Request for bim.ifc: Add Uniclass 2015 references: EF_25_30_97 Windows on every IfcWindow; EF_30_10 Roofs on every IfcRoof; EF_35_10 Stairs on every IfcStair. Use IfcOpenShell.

First a look at what the model holds.

```python
import ifcopenshell

model = ifcopenshell.open("bim.ifc")
print(model.schema)
print("classifications:", [c.Name for c in model.by_type("IfcClassification")])
for ifc_class in ("IfcDoor", "IfcRoof", "IfcStair", "IfcWall", "IfcWindow"):
    print(ifc_class, len(model.by_type(ifc_class)))
```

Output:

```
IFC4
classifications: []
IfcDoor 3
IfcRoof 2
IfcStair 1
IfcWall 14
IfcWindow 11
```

```python
import ifcopenshell
import ifcopenshell.api.classification

model = ifcopenshell.open("bim.ifc")

system = ifcopenshell.api.classification.add_classification(model, classification="Uniclass 2015")

codes = {
    "IfcWindow": ("EF_25_30_97", "Windows"),
    "IfcRoof": ("EF_30_10", "Roofs"),
    "IfcStair": ("EF_35_10", "Stairs"),
}
for ifc_class, (code, name) in codes.items():
    products = model.by_type(ifc_class)
    ifcopenshell.api.classification.add_reference(
        model, products=products, classification=system, identification=code, name=name
    )
    print(code, len(products))

model.write("bim-out.ifc")
```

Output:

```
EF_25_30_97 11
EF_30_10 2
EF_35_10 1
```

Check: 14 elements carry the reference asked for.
